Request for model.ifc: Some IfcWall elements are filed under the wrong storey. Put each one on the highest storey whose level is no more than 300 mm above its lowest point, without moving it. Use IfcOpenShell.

First a look at what the model holds.

```python
import ifcopenshell
import ifcopenshell.util.element
import ifcopenshell.util.placement

model = ifcopenshell.open("model.ifc")
print(model.schema)
for storey in model.by_type("IfcBuildingStorey"):
    level = ifcopenshell.util.placement.get_storey_elevation(storey)
    count = sum(e.is_a("IfcWall") for e in ifcopenshell.util.element.get_contained(storey))
    print(storey.id(), storey.Name, round(level, 3), count, sep=" | ")
```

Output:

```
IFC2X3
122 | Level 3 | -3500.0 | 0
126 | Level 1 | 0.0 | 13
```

```python
import ifcopenshell
import ifcopenshell.api.spatial
import ifcopenshell.geom
import ifcopenshell.util.element
import ifcopenshell.util.placement
import ifcopenshell.util.shape
import ifcopenshell.util.unit

model = ifcopenshell.open("model.ifc")
unit_scale = ifcopenshell.util.unit.calculate_unit_scale(model)
settings = ifcopenshell.geom.settings()

levels = sorted(
    ((ifcopenshell.util.placement.get_storey_elevation(s) * unit_scale, s) for s in model.by_type("IfcBuildingStorey")),
    key=lambda pair: pair[0],
)

for e in model.by_type("IfcWall"):
    current = e.ContainedInStructure[0].RelatingStructure if e.ContainedInStructure else None
    if current is None or not current.is_a("IfcBuildingStorey"):
        continue
    shape = ifcopenshell.geom.create_shape(settings, e)
    bottom = ifcopenshell.util.shape.get_shape_bottom_elevation(shape, shape.geometry)
    below = [s for level, s in levels if level <= bottom + 0.3]
    storey = below[-1] if below else levels[0][1]
    if storey != current:
        # assign_container keeps the world position.
        ifcopenshell.api.spatial.assign_container(model, products=[e], relating_structure=storey)
        print(e.id(), current.Name, "->", storey.Name)

model.write("model_rev.ifc")
```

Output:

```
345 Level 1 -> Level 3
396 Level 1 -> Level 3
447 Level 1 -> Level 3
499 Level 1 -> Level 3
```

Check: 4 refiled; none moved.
